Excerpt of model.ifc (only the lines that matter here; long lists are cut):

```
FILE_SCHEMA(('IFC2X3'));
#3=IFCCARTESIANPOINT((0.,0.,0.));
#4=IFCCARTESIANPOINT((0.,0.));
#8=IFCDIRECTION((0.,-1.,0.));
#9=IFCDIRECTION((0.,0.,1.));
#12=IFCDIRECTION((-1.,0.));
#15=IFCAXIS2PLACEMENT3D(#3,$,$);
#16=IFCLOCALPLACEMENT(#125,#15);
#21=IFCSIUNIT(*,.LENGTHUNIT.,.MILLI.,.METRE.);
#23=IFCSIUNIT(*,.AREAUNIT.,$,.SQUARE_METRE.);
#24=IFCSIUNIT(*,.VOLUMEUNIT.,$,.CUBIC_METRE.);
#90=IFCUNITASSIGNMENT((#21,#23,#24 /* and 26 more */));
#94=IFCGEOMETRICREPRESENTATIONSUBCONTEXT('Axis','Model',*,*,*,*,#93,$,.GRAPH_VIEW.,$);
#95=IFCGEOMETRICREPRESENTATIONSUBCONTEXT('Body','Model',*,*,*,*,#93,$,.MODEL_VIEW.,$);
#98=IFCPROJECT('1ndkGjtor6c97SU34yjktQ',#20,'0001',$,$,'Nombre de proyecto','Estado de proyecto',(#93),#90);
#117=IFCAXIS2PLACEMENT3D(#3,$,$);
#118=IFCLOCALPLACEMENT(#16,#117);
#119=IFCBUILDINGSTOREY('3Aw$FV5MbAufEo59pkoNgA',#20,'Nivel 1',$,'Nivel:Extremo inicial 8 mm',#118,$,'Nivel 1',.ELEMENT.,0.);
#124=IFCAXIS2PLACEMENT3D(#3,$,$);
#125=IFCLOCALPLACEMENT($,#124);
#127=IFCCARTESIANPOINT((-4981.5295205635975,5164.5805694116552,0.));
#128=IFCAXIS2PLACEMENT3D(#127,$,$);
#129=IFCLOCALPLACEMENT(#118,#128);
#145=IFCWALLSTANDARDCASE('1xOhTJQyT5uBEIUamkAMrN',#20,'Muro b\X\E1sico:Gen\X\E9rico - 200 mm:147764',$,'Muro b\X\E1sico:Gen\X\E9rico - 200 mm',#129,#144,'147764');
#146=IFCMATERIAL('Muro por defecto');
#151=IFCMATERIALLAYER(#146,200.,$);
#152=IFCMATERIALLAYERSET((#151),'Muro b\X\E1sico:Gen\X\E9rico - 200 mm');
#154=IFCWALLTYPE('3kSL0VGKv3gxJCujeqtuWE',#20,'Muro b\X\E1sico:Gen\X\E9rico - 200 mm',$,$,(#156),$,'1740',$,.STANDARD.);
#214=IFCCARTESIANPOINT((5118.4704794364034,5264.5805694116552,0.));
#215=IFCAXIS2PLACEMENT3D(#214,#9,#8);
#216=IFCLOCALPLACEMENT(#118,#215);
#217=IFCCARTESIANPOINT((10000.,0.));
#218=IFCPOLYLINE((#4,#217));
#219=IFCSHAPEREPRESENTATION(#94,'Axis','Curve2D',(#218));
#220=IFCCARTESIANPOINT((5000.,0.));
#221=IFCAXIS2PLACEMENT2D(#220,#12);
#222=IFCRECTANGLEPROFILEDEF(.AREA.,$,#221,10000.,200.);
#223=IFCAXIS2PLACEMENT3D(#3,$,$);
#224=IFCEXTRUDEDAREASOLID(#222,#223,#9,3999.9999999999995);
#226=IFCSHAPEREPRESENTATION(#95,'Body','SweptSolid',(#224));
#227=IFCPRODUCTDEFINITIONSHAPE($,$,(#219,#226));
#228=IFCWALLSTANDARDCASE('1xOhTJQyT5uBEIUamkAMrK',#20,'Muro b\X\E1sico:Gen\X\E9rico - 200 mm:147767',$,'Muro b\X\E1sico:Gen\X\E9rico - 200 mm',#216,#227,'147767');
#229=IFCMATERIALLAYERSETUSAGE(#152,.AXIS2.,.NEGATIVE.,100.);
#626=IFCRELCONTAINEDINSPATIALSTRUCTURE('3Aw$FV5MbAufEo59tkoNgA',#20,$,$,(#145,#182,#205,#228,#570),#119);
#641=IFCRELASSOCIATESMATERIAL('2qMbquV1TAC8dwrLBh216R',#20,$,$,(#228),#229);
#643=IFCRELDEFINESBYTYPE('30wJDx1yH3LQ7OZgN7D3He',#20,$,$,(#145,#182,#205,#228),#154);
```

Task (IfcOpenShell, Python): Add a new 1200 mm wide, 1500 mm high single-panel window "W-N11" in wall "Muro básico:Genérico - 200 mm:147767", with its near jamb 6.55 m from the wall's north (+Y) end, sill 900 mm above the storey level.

```python
import numpy as np
import ifcopenshell
import ifcopenshell.api.feature
import ifcopenshell.api.geometry
import ifcopenshell.api.root
import ifcopenshell.api.spatial
import ifcopenshell.api.type
import ifcopenshell.geom
import ifcopenshell.util.element
import ifcopenshell.util.placement
import ifcopenshell.util.representation
import ifcopenshell.util.shape
import ifcopenshell.util.unit

model = ifcopenshell.open("model.ifc")
unit_scale = ifcopenshell.util.unit.calculate_unit_scale(model)
settings = ifcopenshell.geom.settings()


def volume(element):
    """Net volume in cubic metres, openings subtracted."""
    shape = ifcopenshell.geom.create_shape(settings, element)
    return ifcopenshell.util.shape.get_volume(shape.geometry)


wall = model.by_id(228)
storey = ifcopenshell.util.element.get_container(wall, ifc_class="IfcBuildingStorey")
context = ifcopenshell.util.representation.get_context(model, "Model", "Body", "MODEL_VIEW")
before = volume(wall)

width, height, from_end, sill = 1.2, 1.5, 6.55, 0.9  # metres

# The wall runs along its own X axis, and the end named is its -X end.
wall_shape = ifcopenshell.geom.create_shape(settings, wall)
x, y, z = ifcopenshell.util.shape.get_vertices(wall_shape.geometry).T
start = x.min() + from_end
face, thickness = float(y.min()), float(y.max() - y.min())
wall_matrix = ifcopenshell.util.placement.get_local_placement(wall.ObjectPlacement)
level = ifcopenshell.util.placement.get_local_placement(storey.ObjectPlacement)[2, 3]


def in_wall(x, y):
    """Placement at x, y metres in the wall's axes, at sill height."""
    matrix = wall_matrix.copy()
    matrix[:, 3] = wall_matrix @ np.array([x / unit_scale, y / unit_scale, 0.0, 1.0])
    matrix[2, 3] = level + sill / unit_scale
    return matrix


# Opening: a box that overshoots both wall faces by 50 mm.
opening = ifcopenshell.api.root.create_entity(model, ifc_class="IfcOpeningElement")
box = ifcopenshell.api.geometry.add_wall_representation(
    model, context=context, length=width, height=height, thickness=thickness + 0.1
)
ifcopenshell.api.geometry.assign_representation(model, product=opening, representation=box)
ifcopenshell.api.geometry.edit_object_placement(model, product=opening, matrix=in_wall(start, face - 0.05), is_si=False)
ifcopenshell.api.feature.add_feature(model, feature=opening, element=wall)

window = ifcopenshell.api.root.create_entity(model, ifc_class="IfcWindow", name="W-N11")
window.OverallWidth, window.OverallHeight = width / unit_scale, height / unit_scale
body = ifcopenshell.api.geometry.add_window_representation(
    model,
    context=context,
    overall_width=window.OverallWidth,
    overall_height=window.OverallHeight,
    partition_type="SINGLE_PANEL",
)
ifcopenshell.api.geometry.assign_representation(model, product=window, representation=body)
ifcopenshell.api.spatial.assign_container(model, products=[window], relating_structure=storey)
fills = ifcopenshell.api.feature.add_filling(model, opening=opening, element=window)
fills.OwnerHistory = window.OwnerHistory  # required in IFC2X3

# IFC2X3 keeps the operation on the window style.
style = ifcopenshell.api.root.create_entity(model, ifc_class="IfcWindowStyle", name="W-N11")
style.OperationType, style.ConstructionType = "SINGLE_PANEL", "NOTDEFINED"
style.ParameterTakesPrecedence = style.Sizeable = False
ifcopenshell.api.type.assign_type(model, related_objects=[window], relating_type=style)

# Centre the window in the wall's thickness.
ifcopenshell.api.geometry.edit_object_placement(model, product=window, matrix=in_wall(start, face), is_si=False)
window_shape = ifcopenshell.geom.create_shape(settings, window)
depth = ifcopenshell.util.shape.get_vertices(window_shape.geometry)[:, 1]
offset = face + thickness / 2 - (depth.min() + depth.max()) / 2
ifcopenshell.api.geometry.edit_object_placement(model, product=window, matrix=in_wall(start, offset), is_si=False)

after = volume(wall)

print(f"wall volume {before:.3f} -> {after:.3f} m3")

model.write("model_updated.ifc")
```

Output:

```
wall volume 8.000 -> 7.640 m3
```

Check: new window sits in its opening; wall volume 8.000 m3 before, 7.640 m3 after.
